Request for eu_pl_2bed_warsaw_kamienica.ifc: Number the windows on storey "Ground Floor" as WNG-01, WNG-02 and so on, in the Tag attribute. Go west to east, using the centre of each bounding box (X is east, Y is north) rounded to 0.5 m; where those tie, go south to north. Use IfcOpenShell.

First a look at what the model holds.

```python
import ifcopenshell
import ifcopenshell.util.element
import ifcopenshell.util.placement

model = ifcopenshell.open("eu_pl_2bed_warsaw_kamienica.ifc")
print(model.schema)
storey = next(s for s in model.by_type("IfcBuildingStorey") if s.Name == "Ground Floor")
windows = [e for e in ifcopenshell.util.element.get_decomposition(storey) if e.is_a("IfcWindow")]
for e in sorted(windows, key=lambda e: e.id()):
    origin = ifcopenshell.util.placement.get_local_placement(e.ObjectPlacement)[:3, 3]
    print(e.id(), e.Tag, e.Name, origin.round(2) + 0.0, sep=" | ")
```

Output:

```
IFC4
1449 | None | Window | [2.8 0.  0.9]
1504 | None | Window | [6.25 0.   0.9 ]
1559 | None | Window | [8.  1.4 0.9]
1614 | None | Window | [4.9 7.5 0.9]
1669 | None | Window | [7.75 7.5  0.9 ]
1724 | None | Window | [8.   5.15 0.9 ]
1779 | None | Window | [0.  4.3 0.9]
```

```python
import ifcopenshell
import ifcopenshell.geom
import ifcopenshell.util.element
import ifcopenshell.util.shape

model = ifcopenshell.open("eu_pl_2bed_warsaw_kamienica.ifc")
settings = ifcopenshell.geom.settings()
settings.set("use-world-coords", True)


def centre(element):
    shape = ifcopenshell.geom.create_shape(settings, element)
    return ifcopenshell.util.shape.get_bbox_centroid(shape.geometry)


storey = next(s for s in model.by_type("IfcBuildingStorey") if s.Name == "Ground Floor")
windows = [e for e in ifcopenshell.util.element.get_decomposition(storey) if e.is_a("IfcWindow")]

# Insertion points can sit at a corner or the storey origin, so sort by the geometry (in metres).
centres = {e: centre(e) for e in windows}
windows.sort(key=lambda e: (round(centres[e][0] / 0.5), centres[e][1]))

for i, e in enumerate(windows, start=1):
    number = f"WNG-{i:02d}"
    e.Tag = number
    print(e.id(), number)

model.write("eu_pl_2bed_warsaw_kamienica_rev.ifc")
```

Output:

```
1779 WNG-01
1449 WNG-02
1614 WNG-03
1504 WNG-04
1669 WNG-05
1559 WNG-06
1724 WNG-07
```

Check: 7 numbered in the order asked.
